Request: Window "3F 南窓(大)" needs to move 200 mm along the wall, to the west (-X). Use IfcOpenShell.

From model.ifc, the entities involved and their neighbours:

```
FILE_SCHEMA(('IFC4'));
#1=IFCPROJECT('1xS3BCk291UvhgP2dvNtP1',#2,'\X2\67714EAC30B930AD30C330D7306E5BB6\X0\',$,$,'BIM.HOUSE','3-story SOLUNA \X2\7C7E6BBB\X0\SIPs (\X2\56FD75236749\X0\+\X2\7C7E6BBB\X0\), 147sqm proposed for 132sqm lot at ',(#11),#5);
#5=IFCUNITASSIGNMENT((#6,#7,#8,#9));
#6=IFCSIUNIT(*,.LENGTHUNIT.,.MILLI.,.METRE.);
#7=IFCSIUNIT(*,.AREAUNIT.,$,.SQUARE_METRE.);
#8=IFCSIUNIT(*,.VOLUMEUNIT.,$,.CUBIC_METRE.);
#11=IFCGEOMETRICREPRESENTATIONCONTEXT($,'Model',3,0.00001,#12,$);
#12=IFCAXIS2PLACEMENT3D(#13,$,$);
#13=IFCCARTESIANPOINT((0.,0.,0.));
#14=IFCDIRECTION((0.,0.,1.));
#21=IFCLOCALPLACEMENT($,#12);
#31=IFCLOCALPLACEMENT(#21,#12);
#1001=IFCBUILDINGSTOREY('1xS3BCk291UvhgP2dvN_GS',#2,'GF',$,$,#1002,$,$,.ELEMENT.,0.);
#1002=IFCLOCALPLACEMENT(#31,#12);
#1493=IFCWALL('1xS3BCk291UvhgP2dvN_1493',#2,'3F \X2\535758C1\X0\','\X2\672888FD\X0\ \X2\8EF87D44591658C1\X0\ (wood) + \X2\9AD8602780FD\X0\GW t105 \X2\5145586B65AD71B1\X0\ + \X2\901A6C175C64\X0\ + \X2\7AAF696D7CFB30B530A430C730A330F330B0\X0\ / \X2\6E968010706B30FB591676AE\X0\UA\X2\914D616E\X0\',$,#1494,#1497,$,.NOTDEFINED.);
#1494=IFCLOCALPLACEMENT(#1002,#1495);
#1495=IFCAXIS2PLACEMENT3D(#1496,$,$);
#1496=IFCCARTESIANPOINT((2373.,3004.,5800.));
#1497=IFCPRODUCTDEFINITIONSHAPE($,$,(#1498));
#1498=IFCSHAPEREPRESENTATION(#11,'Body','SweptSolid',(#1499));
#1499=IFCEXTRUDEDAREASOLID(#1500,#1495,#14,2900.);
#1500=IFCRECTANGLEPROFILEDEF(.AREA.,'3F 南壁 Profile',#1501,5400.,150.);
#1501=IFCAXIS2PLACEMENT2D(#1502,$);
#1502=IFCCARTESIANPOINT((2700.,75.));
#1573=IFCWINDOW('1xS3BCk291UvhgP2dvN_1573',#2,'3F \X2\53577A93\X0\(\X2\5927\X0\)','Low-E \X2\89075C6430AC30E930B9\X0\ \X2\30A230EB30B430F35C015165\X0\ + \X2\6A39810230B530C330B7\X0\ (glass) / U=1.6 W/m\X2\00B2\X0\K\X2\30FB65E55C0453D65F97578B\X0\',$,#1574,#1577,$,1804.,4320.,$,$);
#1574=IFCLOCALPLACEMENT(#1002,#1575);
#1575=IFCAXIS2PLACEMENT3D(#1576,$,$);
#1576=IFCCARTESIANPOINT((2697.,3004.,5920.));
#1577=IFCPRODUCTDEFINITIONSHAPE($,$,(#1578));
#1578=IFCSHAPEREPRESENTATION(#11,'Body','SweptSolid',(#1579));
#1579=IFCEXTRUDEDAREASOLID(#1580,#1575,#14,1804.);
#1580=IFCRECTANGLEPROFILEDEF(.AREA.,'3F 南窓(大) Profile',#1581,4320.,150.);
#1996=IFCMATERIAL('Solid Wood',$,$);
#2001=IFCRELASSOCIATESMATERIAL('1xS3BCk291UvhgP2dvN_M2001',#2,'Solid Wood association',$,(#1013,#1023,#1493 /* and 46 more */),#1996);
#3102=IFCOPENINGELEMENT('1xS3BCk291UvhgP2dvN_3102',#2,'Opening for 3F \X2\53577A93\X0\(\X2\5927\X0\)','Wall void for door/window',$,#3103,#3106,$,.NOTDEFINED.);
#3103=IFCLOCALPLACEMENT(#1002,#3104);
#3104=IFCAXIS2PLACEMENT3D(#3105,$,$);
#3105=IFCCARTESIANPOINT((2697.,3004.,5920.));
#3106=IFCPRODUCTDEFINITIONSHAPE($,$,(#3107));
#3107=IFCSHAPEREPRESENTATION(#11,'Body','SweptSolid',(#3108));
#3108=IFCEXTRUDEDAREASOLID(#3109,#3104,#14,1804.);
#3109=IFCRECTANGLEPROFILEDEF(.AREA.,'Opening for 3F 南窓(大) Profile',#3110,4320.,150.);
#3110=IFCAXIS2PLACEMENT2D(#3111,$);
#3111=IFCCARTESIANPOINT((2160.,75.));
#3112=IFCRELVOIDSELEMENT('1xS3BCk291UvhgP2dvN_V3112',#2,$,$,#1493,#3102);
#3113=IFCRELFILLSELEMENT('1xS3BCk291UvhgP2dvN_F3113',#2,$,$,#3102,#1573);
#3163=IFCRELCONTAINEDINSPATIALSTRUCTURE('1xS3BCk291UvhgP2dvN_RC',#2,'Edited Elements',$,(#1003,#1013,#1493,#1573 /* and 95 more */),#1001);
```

```python
import ifcopenshell
import ifcopenshell.api.geometry
import ifcopenshell.util.placement
import ifcopenshell.util.unit

model = ifcopenshell.open("model.ifc")
unit_scale = ifcopenshell.util.unit.calculate_unit_scale(model)

window = model.by_id(1573)
opening = window.FillsVoids[0].RelatingOpeningElement
wall = opening.VoidsElements[0].RelatingBuildingElement

wall_matrix = ifcopenshell.util.placement.get_local_placement(wall.ObjectPlacement)
shift = wall_matrix[:3, 0] * -0.2 / unit_scale
before = ifcopenshell.util.placement.get_local_placement(window.ObjectPlacement)[:3, 3].copy()

# The window is not placed relative to its opening, so move both.
for product in (opening, window):
    matrix = ifcopenshell.util.placement.get_local_placement(product.ObjectPlacement)
    matrix[:3, 3] += shift
    ifcopenshell.api.geometry.edit_object_placement(model, product=product, matrix=matrix, is_si=False)

after = ifcopenshell.util.placement.get_local_placement(window.ObjectPlacement)[:3, 3]
print("window moved by", (after - before).round(3) + 0.0)

model.write("model_updated.ifc")
```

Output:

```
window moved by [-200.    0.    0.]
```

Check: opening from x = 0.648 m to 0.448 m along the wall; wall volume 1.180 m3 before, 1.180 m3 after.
